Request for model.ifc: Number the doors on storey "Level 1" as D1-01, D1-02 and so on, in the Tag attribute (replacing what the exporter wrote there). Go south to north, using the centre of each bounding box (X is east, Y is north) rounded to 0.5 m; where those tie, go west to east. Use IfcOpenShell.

First a look at what the model holds.

```python
import ifcopenshell
import ifcopenshell.util.element
import ifcopenshell.util.placement

model = ifcopenshell.open("model.ifc")
print(model.schema)
storey = next(s for s in model.by_type("IfcBuildingStorey") if s.Name == "Level 1")
doors = [e for e in ifcopenshell.util.element.get_decomposition(storey) if e.is_a("IfcDoor")]
for e in sorted(doors, key=lambda e: e.id()):
    origin = ifcopenshell.util.placement.get_local_placement(e.ObjectPlacement)[:3, 3]
    print(e.id(), e.Tag, e.Name, origin.round(2) + 0.0, sep=" | ")
```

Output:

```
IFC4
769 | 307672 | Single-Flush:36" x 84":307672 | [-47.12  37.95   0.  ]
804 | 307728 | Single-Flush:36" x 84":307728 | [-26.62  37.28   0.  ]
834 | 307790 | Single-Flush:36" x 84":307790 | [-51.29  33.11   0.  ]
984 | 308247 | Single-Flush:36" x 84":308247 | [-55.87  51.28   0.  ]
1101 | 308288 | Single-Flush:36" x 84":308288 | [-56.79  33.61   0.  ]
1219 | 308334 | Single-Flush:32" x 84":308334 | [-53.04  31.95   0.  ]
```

```python
import ifcopenshell
import ifcopenshell.geom
import ifcopenshell.util.element
import ifcopenshell.util.shape

model = ifcopenshell.open("model.ifc")
settings = ifcopenshell.geom.settings()
settings.set("use-world-coords", True)


def centre(element):
    shape = ifcopenshell.geom.create_shape(settings, element)
    return ifcopenshell.util.shape.get_bbox_centroid(shape.geometry)


storey = next(s for s in model.by_type("IfcBuildingStorey") if s.Name == "Level 1")
doors = [e for e in ifcopenshell.util.element.get_decomposition(storey) if e.is_a("IfcDoor")]

# Insertion points can sit at a corner or the storey origin, so sort by the geometry (in metres).
centres = {e: centre(e) for e in doors}
doors.sort(key=lambda e: (round(centres[e][1] / 0.5), centres[e][0]))

for i, e in enumerate(doors, start=1):
    number = f"D1-{i:02d}"
    e.Tag = number
    print(e.id(), number)

model.write("model_rev.ifc")
```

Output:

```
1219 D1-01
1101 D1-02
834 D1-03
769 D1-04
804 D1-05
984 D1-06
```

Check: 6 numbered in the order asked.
